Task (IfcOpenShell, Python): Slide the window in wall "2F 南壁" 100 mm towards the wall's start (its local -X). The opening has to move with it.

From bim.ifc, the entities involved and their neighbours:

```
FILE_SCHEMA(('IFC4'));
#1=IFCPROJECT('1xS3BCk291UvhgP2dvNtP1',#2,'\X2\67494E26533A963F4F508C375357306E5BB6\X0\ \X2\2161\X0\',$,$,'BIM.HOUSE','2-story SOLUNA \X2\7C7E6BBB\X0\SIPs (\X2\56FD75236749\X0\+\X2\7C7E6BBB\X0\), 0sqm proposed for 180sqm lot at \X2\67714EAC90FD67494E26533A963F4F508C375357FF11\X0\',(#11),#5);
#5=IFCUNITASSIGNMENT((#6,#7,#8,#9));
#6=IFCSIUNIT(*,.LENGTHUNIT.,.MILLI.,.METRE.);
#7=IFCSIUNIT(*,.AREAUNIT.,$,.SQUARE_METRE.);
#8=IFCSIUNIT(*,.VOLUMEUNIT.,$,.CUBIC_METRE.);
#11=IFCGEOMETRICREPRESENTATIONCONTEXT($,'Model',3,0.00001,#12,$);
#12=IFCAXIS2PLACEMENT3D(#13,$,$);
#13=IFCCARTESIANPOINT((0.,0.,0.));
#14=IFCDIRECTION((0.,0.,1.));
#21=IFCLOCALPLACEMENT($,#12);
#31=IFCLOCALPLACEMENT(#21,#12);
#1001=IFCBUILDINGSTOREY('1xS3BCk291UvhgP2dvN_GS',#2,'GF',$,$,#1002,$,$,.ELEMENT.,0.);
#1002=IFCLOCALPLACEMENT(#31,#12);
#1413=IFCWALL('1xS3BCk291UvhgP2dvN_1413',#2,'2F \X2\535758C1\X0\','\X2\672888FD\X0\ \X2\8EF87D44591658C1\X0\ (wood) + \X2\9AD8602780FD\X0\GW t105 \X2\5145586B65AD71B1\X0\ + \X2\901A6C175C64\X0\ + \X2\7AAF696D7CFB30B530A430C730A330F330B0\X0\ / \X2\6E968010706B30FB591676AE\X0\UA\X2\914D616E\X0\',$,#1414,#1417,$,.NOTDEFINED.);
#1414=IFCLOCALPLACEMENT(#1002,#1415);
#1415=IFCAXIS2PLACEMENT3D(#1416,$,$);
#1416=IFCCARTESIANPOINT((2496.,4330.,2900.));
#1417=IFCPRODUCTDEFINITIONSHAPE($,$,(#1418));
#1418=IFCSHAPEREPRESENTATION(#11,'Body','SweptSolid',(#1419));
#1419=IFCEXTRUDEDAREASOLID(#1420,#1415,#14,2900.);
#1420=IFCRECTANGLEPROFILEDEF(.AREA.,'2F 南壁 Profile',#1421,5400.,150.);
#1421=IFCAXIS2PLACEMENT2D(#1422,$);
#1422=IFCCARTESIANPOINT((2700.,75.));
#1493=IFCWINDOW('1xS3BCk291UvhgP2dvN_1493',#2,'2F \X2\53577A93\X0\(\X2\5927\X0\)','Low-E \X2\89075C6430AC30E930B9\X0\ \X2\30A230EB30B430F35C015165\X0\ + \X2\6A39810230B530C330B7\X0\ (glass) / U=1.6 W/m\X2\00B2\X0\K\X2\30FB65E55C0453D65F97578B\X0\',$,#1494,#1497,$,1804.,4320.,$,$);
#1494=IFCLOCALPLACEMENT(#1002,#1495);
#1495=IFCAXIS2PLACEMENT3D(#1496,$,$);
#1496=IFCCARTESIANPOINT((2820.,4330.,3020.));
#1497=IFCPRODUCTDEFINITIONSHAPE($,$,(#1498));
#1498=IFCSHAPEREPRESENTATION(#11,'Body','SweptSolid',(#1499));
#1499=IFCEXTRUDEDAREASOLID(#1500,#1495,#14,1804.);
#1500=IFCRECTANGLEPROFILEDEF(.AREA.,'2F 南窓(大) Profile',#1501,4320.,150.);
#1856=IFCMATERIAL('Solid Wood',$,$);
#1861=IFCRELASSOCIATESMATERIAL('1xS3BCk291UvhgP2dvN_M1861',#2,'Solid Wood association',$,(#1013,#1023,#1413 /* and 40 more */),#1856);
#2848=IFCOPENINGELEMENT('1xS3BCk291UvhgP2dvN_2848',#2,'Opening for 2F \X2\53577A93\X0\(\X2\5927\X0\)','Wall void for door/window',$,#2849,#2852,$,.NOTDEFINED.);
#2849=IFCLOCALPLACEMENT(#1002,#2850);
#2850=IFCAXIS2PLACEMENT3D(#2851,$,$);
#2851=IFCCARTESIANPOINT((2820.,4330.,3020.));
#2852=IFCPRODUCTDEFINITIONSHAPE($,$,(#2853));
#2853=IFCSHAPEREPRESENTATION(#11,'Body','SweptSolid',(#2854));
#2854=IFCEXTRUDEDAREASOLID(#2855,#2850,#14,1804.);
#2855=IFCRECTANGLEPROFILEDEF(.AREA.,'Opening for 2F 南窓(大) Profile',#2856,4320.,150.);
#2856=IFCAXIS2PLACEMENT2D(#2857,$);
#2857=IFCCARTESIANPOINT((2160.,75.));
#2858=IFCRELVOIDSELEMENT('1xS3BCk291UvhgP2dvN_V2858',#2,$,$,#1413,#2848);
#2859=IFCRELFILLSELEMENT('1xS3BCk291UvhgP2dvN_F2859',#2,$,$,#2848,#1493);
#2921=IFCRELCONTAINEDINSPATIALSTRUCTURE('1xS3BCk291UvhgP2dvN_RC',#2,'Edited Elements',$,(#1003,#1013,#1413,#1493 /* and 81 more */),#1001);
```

```python
import ifcopenshell
import ifcopenshell.api.geometry
import ifcopenshell.util.placement

model = ifcopenshell.open("bim.ifc")

window = model.by_guid("1xS3BCk291UvhgP2dvN_1493")
opening = window.FillsVoids[0].RelatingOpeningElement
wall = opening.VoidsElements[0].RelatingBuildingElement

wall_matrix = ifcopenshell.util.placement.get_local_placement(wall.ObjectPlacement)
shift = wall_matrix[:3, 0] * -100.0
before = ifcopenshell.util.placement.get_local_placement(window.ObjectPlacement)[:3, 3].copy()

# The window is not placed relative to its opening, so move both.
for product in (opening, window):
    matrix = ifcopenshell.util.placement.get_local_placement(product.ObjectPlacement)
    matrix[:3, 3] += shift
    ifcopenshell.api.geometry.edit_object_placement(model, product=product, matrix=matrix, is_si=False)

after = ifcopenshell.util.placement.get_local_placement(window.ObjectPlacement)[:3, 3]
print("window moved by", (after - before).round(3) + 0.0)

model.write("bim_v2.ifc")
```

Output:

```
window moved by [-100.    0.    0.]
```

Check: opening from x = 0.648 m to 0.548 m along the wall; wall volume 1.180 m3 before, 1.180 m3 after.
